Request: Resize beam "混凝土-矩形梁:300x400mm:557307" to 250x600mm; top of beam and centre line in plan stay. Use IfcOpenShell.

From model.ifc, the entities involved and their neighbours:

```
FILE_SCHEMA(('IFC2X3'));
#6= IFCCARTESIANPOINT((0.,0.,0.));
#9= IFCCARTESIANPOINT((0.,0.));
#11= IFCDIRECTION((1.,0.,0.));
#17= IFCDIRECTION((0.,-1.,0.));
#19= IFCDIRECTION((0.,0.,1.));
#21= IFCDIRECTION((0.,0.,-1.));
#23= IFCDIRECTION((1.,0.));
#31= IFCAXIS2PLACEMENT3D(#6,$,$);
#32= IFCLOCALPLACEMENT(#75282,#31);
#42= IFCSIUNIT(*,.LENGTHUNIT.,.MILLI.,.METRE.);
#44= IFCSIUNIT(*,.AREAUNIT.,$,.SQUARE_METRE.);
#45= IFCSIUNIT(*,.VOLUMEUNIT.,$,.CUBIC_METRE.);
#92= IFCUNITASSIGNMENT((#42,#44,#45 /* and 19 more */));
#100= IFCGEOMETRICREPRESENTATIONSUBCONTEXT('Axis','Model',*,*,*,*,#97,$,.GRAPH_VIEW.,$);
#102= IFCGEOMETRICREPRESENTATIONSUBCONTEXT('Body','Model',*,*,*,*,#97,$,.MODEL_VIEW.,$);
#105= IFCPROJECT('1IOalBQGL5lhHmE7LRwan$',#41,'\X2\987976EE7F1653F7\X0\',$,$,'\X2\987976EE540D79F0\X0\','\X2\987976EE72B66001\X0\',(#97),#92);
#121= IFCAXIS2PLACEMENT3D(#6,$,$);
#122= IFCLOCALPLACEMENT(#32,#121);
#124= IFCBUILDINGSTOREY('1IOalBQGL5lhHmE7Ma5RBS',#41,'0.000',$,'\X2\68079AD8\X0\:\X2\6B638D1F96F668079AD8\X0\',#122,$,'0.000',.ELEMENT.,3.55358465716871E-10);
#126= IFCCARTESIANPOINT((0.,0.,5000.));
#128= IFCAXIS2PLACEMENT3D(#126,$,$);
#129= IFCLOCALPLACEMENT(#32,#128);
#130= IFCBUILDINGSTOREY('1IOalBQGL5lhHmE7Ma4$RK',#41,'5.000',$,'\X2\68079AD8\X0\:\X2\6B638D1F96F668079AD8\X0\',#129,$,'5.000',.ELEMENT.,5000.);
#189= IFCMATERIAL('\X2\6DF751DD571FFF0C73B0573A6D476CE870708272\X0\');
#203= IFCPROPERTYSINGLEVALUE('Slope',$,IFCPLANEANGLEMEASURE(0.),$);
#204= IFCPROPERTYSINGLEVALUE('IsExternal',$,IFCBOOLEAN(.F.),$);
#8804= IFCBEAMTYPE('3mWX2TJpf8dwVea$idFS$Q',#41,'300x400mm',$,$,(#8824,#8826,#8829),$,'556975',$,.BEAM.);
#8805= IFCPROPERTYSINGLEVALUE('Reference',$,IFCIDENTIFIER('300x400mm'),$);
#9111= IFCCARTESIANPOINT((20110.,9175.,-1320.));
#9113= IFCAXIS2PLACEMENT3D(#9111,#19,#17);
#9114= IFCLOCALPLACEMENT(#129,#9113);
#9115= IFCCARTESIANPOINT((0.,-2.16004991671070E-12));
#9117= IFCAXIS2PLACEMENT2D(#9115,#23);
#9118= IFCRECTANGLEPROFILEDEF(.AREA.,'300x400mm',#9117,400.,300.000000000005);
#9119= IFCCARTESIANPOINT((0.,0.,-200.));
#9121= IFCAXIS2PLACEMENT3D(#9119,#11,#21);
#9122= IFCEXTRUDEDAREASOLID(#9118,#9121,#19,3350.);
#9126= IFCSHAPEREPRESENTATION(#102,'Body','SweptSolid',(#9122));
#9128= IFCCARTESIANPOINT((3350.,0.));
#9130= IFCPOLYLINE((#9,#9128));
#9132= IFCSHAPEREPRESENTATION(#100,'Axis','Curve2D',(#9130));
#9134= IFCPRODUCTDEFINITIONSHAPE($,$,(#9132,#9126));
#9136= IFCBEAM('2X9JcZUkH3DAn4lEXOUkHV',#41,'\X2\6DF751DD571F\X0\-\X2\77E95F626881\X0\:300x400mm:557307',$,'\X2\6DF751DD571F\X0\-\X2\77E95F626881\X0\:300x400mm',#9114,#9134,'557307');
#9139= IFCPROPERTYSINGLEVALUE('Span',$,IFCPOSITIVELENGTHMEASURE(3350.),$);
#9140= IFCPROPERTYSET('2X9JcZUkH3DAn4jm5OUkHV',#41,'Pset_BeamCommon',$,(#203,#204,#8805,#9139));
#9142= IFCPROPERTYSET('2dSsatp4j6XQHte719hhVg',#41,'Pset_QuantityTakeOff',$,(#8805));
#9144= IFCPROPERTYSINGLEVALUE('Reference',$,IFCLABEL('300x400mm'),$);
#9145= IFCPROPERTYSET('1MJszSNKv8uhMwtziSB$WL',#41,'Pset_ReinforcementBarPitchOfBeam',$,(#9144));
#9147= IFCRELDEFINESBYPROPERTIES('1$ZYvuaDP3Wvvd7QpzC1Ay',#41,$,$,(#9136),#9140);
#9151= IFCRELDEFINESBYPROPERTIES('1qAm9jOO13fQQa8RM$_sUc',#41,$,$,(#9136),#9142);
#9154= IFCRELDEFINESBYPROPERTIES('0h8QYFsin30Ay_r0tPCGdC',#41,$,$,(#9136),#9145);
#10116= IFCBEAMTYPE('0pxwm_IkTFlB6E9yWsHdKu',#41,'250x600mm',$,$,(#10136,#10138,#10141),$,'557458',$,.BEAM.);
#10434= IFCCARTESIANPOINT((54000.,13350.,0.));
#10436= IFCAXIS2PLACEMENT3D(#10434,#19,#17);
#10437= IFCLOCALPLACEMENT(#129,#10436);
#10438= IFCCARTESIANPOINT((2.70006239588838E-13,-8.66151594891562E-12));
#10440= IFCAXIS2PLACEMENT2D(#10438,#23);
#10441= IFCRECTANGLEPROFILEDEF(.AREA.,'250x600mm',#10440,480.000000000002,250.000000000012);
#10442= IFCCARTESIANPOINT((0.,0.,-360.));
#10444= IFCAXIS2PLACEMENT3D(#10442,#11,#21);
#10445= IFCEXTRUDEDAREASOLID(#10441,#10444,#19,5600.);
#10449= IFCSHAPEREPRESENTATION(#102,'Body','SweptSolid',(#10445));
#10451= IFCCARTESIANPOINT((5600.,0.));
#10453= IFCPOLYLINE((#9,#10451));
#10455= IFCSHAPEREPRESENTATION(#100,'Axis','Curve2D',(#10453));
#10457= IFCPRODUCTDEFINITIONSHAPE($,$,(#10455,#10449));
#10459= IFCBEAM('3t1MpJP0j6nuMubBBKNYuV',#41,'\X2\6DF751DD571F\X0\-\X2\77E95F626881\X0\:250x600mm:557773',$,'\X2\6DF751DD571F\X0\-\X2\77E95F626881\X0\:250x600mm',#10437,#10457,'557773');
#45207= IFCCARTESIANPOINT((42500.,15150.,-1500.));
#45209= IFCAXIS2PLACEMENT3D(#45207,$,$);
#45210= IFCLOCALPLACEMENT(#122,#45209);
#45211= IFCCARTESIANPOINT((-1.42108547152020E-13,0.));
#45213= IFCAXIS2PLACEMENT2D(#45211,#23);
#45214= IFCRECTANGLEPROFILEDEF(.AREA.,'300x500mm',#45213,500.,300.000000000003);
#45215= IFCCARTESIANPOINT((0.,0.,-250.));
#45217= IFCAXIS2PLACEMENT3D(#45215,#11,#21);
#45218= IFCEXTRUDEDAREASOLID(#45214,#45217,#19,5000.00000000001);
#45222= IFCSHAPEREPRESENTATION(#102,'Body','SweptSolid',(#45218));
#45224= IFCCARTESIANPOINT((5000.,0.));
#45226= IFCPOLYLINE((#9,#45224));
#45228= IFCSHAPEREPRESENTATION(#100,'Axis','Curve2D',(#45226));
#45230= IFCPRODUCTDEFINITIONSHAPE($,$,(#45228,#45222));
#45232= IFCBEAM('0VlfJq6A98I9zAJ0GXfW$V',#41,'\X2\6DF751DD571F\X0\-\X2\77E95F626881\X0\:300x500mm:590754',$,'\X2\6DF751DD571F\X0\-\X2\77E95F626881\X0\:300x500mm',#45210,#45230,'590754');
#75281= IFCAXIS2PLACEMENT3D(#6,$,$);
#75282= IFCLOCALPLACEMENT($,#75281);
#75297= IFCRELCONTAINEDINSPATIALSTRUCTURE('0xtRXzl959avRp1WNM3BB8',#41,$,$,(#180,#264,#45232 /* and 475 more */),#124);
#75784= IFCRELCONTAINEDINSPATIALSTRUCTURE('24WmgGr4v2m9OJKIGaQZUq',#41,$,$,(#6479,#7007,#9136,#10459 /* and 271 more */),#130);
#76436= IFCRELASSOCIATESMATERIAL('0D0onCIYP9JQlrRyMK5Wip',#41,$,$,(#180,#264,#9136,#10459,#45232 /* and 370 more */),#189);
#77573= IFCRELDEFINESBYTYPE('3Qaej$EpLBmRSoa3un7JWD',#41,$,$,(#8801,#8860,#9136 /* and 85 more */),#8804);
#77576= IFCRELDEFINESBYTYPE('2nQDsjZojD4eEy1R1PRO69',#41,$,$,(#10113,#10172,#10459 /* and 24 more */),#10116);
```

```python
import ifcopenshell
import ifcopenshell.api.pset
import ifcopenshell.api.type
import ifcopenshell.util.element
import ifcopenshell.util.representation

model = ifcopenshell.open("model.ifc")

member = model.by_id(9136)
source = next(p for p in model.by_type("IfcRectangleProfileDef") if p.ProfileName == "250x600mm")

body = ifcopenshell.util.representation.get_representation(member, "Model", "Body")
solid = body.Items[0]
old_profile = solid.SweptArea

# Copy the section's sizes but keep this member's own profile position.
profile = ifcopenshell.util.element.copy(model, source)
# Profiles are centred, so shift by half the change in depth to hold the top.
shift = (old_profile.XDim - profile.XDim) / 2
x, y = old_profile.Position.Location.Coordinates
up = (-1.0, 0.0)  # upwards, in the solid's own plane
location = model.createIfcCartesianPoint((x + up[0] * shift, y + up[1] * shift))
profile.Position = model.createIfcAxis2Placement2D(location, old_profile.Position.RefDirection)
solid.SweptArea = profile
if not model.get_total_inverses(old_profile):
    ifcopenshell.util.element.remove_deep2(model, old_profile)

new_type = model.by_guid("0pxwm_IkTFlB6E9yWsHdKu")
ifcopenshell.api.type.assign_type(
    model, related_objects=[member], relating_type=new_type, should_map_representations=False
)
member.Name = member.Name.replace("300x400mm", "250x600mm")
member.ObjectType = "混凝土-矩形梁:250x600mm"
pset = model.by_id(ifcopenshell.util.element.get_pset(member, "Pset_BeamCommon", should_inherit=False)["id"])
ifcopenshell.api.pset.edit_pset(model, pset=pset, properties={"Reference": "250x600mm"})
pset = model.by_id(ifcopenshell.util.element.get_pset(member, "Pset_QuantityTakeOff", should_inherit=False)["id"])
ifcopenshell.api.pset.edit_pset(model, pset=pset, properties={"Reference": "250x600mm"})
pset = model.by_id(ifcopenshell.util.element.get_pset(member, "Pset_ReinforcementBarPitchOfBeam", should_inherit=False)["id"])
ifcopenshell.api.pset.edit_pset(model, pset=pset, properties={"Reference": "250x600mm"})

print(solid.SweptArea)

model.write("model_updated.ifc")
```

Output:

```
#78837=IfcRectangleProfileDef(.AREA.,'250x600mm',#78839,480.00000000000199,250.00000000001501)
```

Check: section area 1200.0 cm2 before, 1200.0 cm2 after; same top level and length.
